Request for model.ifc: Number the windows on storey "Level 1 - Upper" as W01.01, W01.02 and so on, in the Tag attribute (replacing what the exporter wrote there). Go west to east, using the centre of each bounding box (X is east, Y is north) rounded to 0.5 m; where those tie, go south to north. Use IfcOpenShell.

First a look at what the model holds.

```python
import ifcopenshell
import ifcopenshell.util.element
import ifcopenshell.util.placement

model = ifcopenshell.open("model.ifc")
print(model.schema)
storey = next(s for s in model.by_type("IfcBuildingStorey") if s.Name == "Level 1 - Upper")
windows = [e for e in ifcopenshell.util.element.get_decomposition(storey) if e.is_a("IfcWindow")]
for e in sorted(windows, key=lambda e: e.id()):
    origin = ifcopenshell.util.placement.get_local_placement(e.ObjectPlacement)[:3, 3]
    print(e.id(), e.Tag, e.Name, origin.round(2) + 0.0, sep=" | ")
```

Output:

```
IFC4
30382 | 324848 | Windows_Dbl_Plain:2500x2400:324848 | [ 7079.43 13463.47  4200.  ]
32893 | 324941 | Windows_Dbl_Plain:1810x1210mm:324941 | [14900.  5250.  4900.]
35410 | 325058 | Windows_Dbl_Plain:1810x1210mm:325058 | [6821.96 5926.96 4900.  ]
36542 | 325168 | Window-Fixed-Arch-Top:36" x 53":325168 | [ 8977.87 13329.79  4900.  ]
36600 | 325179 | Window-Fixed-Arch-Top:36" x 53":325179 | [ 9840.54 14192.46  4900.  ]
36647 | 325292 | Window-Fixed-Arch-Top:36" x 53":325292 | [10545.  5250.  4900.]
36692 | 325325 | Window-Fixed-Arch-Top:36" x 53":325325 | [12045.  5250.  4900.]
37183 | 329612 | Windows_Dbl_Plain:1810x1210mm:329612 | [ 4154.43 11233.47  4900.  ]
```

```python
import ifcopenshell
import ifcopenshell.geom
import ifcopenshell.util.element
import ifcopenshell.util.shape

model = ifcopenshell.open("model.ifc")
settings = ifcopenshell.geom.settings()
settings.set("use-world-coords", True)


def centre(element):
    shape = ifcopenshell.geom.create_shape(settings, element)
    return ifcopenshell.util.shape.get_bbox_centroid(shape.geometry)


storey = next(s for s in model.by_type("IfcBuildingStorey") if s.Name == "Level 1 - Upper")
windows = [e for e in ifcopenshell.util.element.get_decomposition(storey) if e.is_a("IfcWindow")]

# Insertion points can sit at a corner or the storey origin, so sort by the geometry (in metres).
centres = {e: centre(e) for e in windows}
windows.sort(key=lambda e: (round(centres[e][0] / 0.5), centres[e][1]))

for i, e in enumerate(windows, start=1):
    number = f"W01.{i:02d}"
    e.Tag = number
    print(e.id(), number)

model.write("model_edited.ifc")
```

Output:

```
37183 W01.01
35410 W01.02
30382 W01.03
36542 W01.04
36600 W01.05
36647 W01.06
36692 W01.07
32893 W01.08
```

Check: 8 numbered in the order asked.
